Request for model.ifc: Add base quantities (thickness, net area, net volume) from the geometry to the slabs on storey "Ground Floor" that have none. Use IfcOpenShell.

First a look at what the model holds.

```python
import ifcopenshell
import ifcopenshell.util.element
import ifcopenshell.util.unit

model = ifcopenshell.open("model.ifc")
print(model.schema)
for unit_type in ("LENGTHUNIT", "AREAUNIT", "VOLUMEUNIT"):
    print(unit_type, ifcopenshell.util.unit.calculate_unit_scale(model, unit_type))
storey = next(s for s in model.by_type("IfcBuildingStorey") if s.Name == "Ground Floor")
slabs = [e for e in ifcopenshell.util.element.get_decomposition(storey) if e.is_a("IfcSlab")]
for e in sorted(slabs, key=lambda e: e.id()):
    print(e.id(), e.is_a(), e.Name, list(ifcopenshell.util.element.get_psets(e, qtos_only=True)), sep=" | ")
```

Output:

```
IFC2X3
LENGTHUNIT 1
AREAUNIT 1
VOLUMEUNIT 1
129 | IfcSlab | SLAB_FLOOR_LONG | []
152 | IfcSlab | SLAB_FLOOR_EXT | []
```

```python
import ifcopenshell
import ifcopenshell.api.pset
import ifcopenshell.geom
import ifcopenshell.util.element
import ifcopenshell.util.shape
import ifcopenshell.util.unit

model = ifcopenshell.open("model.ifc")
unit_scale = ifcopenshell.util.unit.calculate_unit_scale(model)
area_scale = ifcopenshell.util.unit.calculate_unit_scale(model, "AREAUNIT")
volume_scale = ifcopenshell.util.unit.calculate_unit_scale(model, "VOLUMEUNIT")
settings = ifcopenshell.geom.settings()

storey = next(s for s in model.by_type("IfcBuildingStorey") if s.Name == "Ground Floor")
slabs = [e for e in ifcopenshell.util.element.get_decomposition(storey) if e.is_a("IfcSlab")]

for e in sorted(slabs, key=lambda e: e.id()):
    if ifcopenshell.util.element.get_psets(e, qtos_only=True, should_inherit=False):
        continue
    # Geometry comes back in metres, in the element's own axes.
    shape = ifcopenshell.geom.create_shape(settings, e)
    values = {
        "Width": ifcopenshell.util.shape.get_z(shape.geometry) / unit_scale,
        "NetArea": ifcopenshell.util.shape.get_footprint_area(shape.geometry) / area_scale,
        "NetVolume": ifcopenshell.util.shape.get_volume(shape.geometry) / volume_scale,
    }
    qto = ifcopenshell.api.pset.add_qto(model, product=e, name="BaseQuantities")
    ifcopenshell.api.pset.edit_qto(model, qto=qto, properties=values)
    print(e.id(), {k: round(v, 3) for k, v in values.items()})

model.write("model_updated.ifc")
```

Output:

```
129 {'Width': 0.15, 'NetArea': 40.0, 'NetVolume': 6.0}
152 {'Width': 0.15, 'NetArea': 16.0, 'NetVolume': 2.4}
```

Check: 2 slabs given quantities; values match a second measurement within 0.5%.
